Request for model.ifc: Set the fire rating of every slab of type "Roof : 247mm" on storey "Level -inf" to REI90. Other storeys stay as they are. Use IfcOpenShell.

First a look at what the model holds.

```python
import ifcopenshell
import ifcopenshell.util.element

model = ifcopenshell.open("model.ifc")
print(model.schema)
storey = next(s for s in model.by_type("IfcBuildingStorey") if s.Name == "Level -inf")
slabs = [e for e in ifcopenshell.util.element.get_decomposition(storey) if e.is_a("IfcSlab")]
seen = {}
for e in slabs:
    element_type = ifcopenshell.util.element.get_type(e)
    key = (element_type.Name if element_type != e and element_type else None, ifcopenshell.util.element.get_pset(e, "Pset_SlabCommon", "FireRating"))
    seen[key] = seen.get(key, 0) + 1
for (name, value), count in sorted(seen.items(), key=str):
    print(count, "x", name, "|", value)
```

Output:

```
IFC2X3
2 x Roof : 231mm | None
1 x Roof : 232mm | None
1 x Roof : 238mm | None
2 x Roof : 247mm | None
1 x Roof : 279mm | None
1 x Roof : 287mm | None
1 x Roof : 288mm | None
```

```python
import ifcopenshell
import ifcopenshell.api.pset
import ifcopenshell.util.element

model = ifcopenshell.open("model.ifc")

storey = next(s for s in model.by_type("IfcBuildingStorey") if s.Name == "Level -inf")
slabs = [e for e in ifcopenshell.util.element.get_decomposition(storey) if e.is_a("IfcSlab")]

count = 0
for e in slabs:
    element_type = ifcopenshell.util.element.get_type(e)
    if element_type in (None, e) or element_type.Name != "Roof : 247mm":
        continue
    # add_pset returns the element's existing set when there is one.
    pset = ifcopenshell.api.pset.add_pset(model, product=e, name="Pset_SlabCommon")
    ifcopenshell.api.pset.edit_pset(model, pset=pset, properties={"FireRating": "REI90"})
    count += 1

print(count, "slabs updated")

model.write("model-out.ifc")
```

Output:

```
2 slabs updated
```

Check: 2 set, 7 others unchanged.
